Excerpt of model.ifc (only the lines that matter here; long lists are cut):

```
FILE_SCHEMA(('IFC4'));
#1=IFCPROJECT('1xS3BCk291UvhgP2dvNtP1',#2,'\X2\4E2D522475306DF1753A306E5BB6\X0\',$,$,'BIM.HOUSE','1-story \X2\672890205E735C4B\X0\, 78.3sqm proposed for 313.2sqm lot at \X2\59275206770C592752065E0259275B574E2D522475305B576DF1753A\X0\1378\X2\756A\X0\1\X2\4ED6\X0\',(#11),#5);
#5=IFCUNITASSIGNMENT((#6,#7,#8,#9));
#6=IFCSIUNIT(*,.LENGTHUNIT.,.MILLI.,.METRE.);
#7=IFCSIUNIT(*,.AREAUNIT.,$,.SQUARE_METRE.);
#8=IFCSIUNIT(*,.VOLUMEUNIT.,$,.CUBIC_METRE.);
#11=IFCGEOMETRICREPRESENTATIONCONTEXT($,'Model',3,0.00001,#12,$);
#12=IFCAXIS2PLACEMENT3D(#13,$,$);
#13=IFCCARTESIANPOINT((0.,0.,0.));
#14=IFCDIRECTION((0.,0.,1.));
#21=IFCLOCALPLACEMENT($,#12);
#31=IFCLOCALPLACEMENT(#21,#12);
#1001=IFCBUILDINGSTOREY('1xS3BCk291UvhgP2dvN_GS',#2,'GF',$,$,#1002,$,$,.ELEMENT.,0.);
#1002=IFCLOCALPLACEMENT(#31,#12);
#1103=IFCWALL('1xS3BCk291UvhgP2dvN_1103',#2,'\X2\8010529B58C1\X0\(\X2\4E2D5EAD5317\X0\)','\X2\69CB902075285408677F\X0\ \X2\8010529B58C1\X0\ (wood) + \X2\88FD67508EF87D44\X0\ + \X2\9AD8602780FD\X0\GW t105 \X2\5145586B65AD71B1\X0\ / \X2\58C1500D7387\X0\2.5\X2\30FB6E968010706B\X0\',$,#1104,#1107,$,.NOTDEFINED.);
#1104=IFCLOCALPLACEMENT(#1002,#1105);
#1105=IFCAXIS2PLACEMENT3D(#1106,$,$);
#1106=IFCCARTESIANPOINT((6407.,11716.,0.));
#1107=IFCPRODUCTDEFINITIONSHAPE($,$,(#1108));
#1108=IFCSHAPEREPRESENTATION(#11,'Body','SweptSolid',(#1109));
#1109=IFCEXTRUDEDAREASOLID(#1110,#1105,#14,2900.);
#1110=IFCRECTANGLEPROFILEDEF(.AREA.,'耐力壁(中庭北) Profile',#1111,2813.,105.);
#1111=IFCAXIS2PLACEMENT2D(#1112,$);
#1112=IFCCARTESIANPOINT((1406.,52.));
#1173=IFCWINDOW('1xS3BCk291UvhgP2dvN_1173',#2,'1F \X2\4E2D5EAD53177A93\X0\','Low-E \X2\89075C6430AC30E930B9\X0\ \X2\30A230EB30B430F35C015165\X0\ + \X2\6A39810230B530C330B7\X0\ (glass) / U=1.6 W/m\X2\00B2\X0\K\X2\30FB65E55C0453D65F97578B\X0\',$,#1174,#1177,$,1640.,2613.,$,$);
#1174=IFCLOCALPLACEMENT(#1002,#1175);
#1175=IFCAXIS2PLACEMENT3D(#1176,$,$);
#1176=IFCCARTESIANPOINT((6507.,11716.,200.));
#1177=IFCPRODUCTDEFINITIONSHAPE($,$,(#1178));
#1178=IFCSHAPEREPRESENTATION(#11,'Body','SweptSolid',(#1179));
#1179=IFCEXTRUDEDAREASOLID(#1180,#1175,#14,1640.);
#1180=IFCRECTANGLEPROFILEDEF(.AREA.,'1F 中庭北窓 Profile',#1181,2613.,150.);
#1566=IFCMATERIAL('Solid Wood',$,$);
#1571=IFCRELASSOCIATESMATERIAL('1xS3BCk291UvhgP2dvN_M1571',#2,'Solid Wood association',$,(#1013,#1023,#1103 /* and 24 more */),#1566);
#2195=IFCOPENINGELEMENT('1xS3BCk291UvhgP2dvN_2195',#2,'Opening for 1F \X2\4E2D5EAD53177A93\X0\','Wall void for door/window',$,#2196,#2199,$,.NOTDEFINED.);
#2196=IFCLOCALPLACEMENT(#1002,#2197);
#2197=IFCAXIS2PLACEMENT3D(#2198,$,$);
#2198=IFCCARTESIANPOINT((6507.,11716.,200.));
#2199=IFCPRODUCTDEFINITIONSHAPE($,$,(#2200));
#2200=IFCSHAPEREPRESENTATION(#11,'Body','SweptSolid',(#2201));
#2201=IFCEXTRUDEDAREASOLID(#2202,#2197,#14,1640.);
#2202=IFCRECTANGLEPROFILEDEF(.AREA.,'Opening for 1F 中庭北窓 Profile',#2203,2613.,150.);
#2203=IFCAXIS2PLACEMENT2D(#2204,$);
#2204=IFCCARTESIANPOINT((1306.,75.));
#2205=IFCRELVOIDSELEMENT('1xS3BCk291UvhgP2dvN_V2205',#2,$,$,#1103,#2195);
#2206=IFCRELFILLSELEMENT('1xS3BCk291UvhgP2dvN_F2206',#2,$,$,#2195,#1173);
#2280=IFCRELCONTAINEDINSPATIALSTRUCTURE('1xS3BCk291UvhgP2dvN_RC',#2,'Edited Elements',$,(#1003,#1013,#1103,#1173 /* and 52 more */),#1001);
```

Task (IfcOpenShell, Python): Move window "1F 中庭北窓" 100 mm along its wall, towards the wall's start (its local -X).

```python
import ifcopenshell
import ifcopenshell.api.geometry
import ifcopenshell.util.placement
import ifcopenshell.util.unit

model = ifcopenshell.open("model.ifc")
unit_scale = ifcopenshell.util.unit.calculate_unit_scale(model)

window = model.by_guid("1xS3BCk291UvhgP2dvN_1173")
opening = window.FillsVoids[0].RelatingOpeningElement
wall = opening.VoidsElements[0].RelatingBuildingElement

wall_matrix = ifcopenshell.util.placement.get_local_placement(wall.ObjectPlacement)
shift = wall_matrix[:3, 0] * -0.1 / unit_scale
before = ifcopenshell.util.placement.get_local_placement(window.ObjectPlacement)[:3, 3].copy()

# The window is not placed relative to its opening, so move both.
for product in (opening, window):
    matrix = ifcopenshell.util.placement.get_local_placement(product.ObjectPlacement)
    matrix[:3, 3] += shift
    ifcopenshell.api.geometry.edit_object_placement(model, product=product, matrix=matrix, is_si=False)

after = ifcopenshell.util.placement.get_local_placement(window.ObjectPlacement)[:3, 3]
print("window moved by", (after - before).round(3) + 0.0)

model.write("model_updated.ifc")
```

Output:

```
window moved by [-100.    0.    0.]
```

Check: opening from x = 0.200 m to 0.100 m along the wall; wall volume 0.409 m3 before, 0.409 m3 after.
